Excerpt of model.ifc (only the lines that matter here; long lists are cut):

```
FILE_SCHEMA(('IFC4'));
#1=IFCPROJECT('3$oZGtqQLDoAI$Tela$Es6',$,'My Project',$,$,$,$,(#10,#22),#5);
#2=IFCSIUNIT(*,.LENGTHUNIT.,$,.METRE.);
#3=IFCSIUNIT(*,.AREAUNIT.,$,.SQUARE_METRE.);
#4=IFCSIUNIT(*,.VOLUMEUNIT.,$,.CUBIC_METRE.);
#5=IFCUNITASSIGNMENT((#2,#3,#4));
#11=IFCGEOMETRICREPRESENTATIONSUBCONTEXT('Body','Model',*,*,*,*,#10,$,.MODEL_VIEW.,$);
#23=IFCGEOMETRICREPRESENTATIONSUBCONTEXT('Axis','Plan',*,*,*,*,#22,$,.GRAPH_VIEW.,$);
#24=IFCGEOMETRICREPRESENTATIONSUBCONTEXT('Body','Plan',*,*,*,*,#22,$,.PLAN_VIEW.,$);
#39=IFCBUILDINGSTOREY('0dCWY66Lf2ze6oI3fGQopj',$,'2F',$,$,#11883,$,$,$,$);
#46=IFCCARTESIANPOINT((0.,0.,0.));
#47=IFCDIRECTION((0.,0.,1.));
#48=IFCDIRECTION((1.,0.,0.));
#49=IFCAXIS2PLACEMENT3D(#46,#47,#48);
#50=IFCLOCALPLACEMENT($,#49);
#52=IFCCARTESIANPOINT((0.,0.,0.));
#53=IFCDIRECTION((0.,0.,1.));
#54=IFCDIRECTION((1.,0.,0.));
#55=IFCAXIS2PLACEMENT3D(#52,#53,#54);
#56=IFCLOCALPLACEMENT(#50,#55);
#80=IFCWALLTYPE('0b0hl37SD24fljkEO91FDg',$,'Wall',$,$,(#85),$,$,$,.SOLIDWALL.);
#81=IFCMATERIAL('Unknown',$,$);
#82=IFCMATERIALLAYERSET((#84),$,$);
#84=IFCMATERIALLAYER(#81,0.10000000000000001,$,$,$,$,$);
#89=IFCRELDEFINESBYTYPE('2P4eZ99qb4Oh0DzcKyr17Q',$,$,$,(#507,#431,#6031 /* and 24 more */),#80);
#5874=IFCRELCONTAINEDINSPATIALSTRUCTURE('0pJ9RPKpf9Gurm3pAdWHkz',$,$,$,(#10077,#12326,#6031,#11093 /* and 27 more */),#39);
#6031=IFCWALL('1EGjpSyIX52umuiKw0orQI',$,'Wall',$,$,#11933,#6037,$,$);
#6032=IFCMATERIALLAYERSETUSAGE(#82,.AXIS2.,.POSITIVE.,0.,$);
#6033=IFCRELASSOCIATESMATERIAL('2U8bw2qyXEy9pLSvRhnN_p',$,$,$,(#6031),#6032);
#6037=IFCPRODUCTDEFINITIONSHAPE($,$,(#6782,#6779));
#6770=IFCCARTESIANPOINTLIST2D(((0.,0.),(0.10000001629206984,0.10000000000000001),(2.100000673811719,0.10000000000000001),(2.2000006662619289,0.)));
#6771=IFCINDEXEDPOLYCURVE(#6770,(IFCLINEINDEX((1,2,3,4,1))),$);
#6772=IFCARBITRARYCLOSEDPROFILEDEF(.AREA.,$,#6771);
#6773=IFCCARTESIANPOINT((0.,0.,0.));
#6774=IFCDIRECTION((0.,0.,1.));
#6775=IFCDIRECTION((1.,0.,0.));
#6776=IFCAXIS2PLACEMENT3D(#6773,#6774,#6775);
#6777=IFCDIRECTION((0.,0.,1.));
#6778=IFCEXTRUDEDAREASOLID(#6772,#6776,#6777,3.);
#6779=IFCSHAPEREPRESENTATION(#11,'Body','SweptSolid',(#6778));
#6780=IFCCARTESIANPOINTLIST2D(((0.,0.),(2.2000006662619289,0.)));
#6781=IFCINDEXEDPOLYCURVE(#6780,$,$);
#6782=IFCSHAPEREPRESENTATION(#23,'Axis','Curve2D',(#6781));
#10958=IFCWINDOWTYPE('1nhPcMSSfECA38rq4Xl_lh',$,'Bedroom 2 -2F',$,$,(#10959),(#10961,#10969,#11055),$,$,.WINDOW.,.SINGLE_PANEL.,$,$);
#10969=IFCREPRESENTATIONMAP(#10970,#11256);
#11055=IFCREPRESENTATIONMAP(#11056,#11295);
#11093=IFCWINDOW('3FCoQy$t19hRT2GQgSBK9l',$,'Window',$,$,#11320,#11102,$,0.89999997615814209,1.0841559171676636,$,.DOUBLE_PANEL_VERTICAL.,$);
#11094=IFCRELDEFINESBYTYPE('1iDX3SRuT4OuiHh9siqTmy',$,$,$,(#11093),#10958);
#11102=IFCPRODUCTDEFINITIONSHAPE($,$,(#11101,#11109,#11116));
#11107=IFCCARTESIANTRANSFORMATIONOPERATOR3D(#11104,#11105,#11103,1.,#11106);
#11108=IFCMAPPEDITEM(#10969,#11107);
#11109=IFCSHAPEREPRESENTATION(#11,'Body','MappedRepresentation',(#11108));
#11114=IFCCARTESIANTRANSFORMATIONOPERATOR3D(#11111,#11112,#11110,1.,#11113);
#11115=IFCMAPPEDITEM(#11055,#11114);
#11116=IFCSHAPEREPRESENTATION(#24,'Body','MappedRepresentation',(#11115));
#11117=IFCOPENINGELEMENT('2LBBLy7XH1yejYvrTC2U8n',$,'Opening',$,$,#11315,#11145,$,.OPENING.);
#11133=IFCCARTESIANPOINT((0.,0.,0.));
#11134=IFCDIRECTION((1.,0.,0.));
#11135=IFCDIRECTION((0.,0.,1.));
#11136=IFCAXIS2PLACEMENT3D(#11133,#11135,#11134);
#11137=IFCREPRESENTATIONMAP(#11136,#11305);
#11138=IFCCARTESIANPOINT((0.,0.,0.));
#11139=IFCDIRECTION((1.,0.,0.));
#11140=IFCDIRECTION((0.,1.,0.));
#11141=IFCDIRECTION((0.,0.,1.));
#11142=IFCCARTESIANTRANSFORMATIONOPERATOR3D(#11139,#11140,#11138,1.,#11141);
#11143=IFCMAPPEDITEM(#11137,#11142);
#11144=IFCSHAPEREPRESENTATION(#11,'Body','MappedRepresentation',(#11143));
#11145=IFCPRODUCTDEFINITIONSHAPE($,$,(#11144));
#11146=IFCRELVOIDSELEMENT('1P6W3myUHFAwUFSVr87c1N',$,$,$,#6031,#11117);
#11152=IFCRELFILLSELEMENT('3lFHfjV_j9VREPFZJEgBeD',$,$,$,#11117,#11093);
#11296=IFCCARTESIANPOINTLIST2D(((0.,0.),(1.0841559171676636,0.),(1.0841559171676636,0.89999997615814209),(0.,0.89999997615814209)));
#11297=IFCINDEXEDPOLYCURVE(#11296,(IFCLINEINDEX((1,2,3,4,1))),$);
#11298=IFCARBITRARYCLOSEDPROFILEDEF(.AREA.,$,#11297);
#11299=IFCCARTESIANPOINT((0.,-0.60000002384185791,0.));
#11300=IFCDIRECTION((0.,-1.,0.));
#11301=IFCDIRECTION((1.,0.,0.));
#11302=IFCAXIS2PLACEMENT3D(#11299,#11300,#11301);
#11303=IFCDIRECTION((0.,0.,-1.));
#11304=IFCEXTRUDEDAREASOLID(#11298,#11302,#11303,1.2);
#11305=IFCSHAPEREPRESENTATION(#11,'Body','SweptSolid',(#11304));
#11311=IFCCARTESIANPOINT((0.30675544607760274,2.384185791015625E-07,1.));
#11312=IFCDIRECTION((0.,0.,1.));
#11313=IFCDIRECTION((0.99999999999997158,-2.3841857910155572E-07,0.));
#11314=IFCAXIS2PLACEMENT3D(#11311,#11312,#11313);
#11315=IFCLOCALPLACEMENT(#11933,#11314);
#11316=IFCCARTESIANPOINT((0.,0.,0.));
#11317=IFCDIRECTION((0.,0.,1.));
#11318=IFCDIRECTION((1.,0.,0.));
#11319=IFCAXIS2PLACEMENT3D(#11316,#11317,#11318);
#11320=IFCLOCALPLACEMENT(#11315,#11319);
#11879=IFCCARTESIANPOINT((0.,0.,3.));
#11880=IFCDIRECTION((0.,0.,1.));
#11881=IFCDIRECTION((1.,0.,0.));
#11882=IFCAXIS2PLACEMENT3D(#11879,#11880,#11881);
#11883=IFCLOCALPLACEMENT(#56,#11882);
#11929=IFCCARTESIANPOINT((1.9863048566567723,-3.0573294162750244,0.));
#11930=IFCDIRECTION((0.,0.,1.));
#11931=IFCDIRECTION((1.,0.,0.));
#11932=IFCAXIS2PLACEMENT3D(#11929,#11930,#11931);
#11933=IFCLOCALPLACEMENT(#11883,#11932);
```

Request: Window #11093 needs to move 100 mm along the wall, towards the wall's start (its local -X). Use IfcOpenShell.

```python
import ifcopenshell
import ifcopenshell.api.geometry
import ifcopenshell.util.placement
import ifcopenshell.util.unit

model = ifcopenshell.open("model.ifc")
unit_scale = ifcopenshell.util.unit.calculate_unit_scale(model)

window = model.by_guid("3FCoQy$t19hRT2GQgSBK9l")
opening = window.FillsVoids[0].RelatingOpeningElement
wall = opening.VoidsElements[0].RelatingBuildingElement

wall_matrix = ifcopenshell.util.placement.get_local_placement(wall.ObjectPlacement)
shift = wall_matrix[:3, 0] * -0.1 / unit_scale
before = ifcopenshell.util.placement.get_local_placement(window.ObjectPlacement)[:3, 3].copy()

# The window is placed relative to its opening, so it follows when the opening moves.
matrix = ifcopenshell.util.placement.get_local_placement(opening.ObjectPlacement)
matrix[:3, 3] += shift
ifcopenshell.api.geometry.edit_object_placement(
    model, product=opening, matrix=matrix, is_si=False, should_transform_children=True
)

after = ifcopenshell.util.placement.get_local_placement(window.ObjectPlacement)[:3, 3]
print("window moved by", (after - before).round(3) + 0.0)

model.write("model_updated.ifc")
```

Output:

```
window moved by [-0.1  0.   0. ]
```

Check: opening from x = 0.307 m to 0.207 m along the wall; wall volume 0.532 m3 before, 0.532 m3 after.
